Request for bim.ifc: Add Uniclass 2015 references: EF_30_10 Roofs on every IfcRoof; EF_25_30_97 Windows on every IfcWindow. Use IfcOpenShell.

First a look at what the model holds.

```python
import ifcopenshell

model = ifcopenshell.open("bim.ifc")
print(model.schema)
print("classifications:", [c.Name for c in model.by_type("IfcClassification")])
for ifc_class in ("IfcDoor", "IfcRoof", "IfcStair", "IfcWall", "IfcWindow"):
    print(ifc_class, len(model.by_type(ifc_class)))
```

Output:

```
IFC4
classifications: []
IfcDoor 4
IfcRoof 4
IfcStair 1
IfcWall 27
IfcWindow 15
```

```python
import ifcopenshell
import ifcopenshell.api.classification

model = ifcopenshell.open("bim.ifc")

system = ifcopenshell.api.classification.add_classification(model, classification="Uniclass 2015")

codes = {
    "IfcRoof": ("EF_30_10", "Roofs"),
    "IfcWindow": ("EF_25_30_97", "Windows"),
}
for ifc_class, (code, name) in codes.items():
    products = model.by_type(ifc_class)
    ifcopenshell.api.classification.add_reference(
        model, products=products, classification=system, identification=code, name=name
    )
    print(code, len(products))

model.write("bim_v2.ifc")
```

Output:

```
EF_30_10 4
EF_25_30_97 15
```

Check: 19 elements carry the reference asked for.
